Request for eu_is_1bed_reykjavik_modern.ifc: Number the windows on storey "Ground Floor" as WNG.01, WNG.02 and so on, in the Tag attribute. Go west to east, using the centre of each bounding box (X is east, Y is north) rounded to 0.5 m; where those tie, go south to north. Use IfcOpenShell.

First a look at what the model holds.

```python
import ifcopenshell
import ifcopenshell.util.element
import ifcopenshell.util.placement

model = ifcopenshell.open("eu_is_1bed_reykjavik_modern.ifc")
print(model.schema)
storey = next(s for s in model.by_type("IfcBuildingStorey") if s.Name == "Ground Floor")
windows = [e for e in ifcopenshell.util.element.get_decomposition(storey) if e.is_a("IfcWindow")]
for e in sorted(windows, key=lambda e: e.id()):
    origin = ifcopenshell.util.placement.get_local_placement(e.ObjectPlacement)[:3, 3]
    print(e.id(), e.Tag, e.Name, origin.round(2) + 0.0, sep=" | ")
```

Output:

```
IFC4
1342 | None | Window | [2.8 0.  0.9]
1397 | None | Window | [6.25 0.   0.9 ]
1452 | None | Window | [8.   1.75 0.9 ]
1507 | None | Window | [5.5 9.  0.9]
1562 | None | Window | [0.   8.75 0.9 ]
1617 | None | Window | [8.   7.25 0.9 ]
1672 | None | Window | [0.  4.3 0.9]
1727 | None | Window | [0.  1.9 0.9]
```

```python
import ifcopenshell
import ifcopenshell.geom
import ifcopenshell.util.element
import ifcopenshell.util.shape

model = ifcopenshell.open("eu_is_1bed_reykjavik_modern.ifc")
settings = ifcopenshell.geom.settings()
settings.set("use-world-coords", True)


def centre(element):
    shape = ifcopenshell.geom.create_shape(settings, element)
    return ifcopenshell.util.shape.get_bbox_centroid(shape.geometry)


storey = next(s for s in model.by_type("IfcBuildingStorey") if s.Name == "Ground Floor")
windows = [e for e in ifcopenshell.util.element.get_decomposition(storey) if e.is_a("IfcWindow")]

# Insertion points can sit at a corner or the storey origin, so sort by the geometry (in metres).
centres = {e: centre(e) for e in windows}
windows.sort(key=lambda e: (round(centres[e][0] / 0.5), centres[e][1]))

for i, e in enumerate(windows, start=1):
    number = f"WNG.{i:02d}"
    e.Tag = number
    print(e.id(), number)

model.write("eu_is_1bed_reykjavik_modern_edited.ifc")
```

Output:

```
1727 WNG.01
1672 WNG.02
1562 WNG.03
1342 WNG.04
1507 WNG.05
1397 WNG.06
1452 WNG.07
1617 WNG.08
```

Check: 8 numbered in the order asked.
